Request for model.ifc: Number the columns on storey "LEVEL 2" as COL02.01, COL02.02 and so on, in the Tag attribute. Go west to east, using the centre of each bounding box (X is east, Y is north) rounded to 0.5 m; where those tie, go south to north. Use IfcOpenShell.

First a look at what the model holds.

```python
import ifcopenshell
import ifcopenshell.util.element
import ifcopenshell.util.placement

model = ifcopenshell.open("model.ifc")
print(model.schema)
storey = next(s for s in model.by_type("IfcBuildingStorey") if s.Name == "LEVEL 2")
columns = [e for e in ifcopenshell.util.element.get_decomposition(storey) if e.is_a("IfcColumn")]
for e in sorted(columns, key=lambda e: e.id()):
    origin = ifcopenshell.util.placement.get_local_placement(e.ObjectPlacement)[:3, 3]
    print(e.id(), e.Tag, e.Name, origin.round(2) + 0.0, sep=" | ")
```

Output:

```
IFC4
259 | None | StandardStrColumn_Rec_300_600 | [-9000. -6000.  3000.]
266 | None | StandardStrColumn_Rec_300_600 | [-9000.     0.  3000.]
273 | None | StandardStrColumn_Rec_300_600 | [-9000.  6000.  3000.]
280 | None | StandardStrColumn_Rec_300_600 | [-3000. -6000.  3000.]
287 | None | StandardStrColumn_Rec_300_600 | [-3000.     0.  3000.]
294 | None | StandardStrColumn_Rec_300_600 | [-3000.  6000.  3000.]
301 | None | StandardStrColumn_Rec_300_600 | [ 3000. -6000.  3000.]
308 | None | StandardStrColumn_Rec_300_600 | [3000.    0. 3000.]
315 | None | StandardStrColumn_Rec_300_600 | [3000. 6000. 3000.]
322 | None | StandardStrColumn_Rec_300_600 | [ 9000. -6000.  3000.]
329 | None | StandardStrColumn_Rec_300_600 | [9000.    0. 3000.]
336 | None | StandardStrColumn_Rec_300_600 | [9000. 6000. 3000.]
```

```python
import ifcopenshell
import ifcopenshell.geom
import ifcopenshell.util.element
import ifcopenshell.util.shape

model = ifcopenshell.open("model.ifc")
settings = ifcopenshell.geom.settings()
settings.set("use-world-coords", True)


def centre(element):
    shape = ifcopenshell.geom.create_shape(settings, element)
    return ifcopenshell.util.shape.get_bbox_centroid(shape.geometry)


storey = next(s for s in model.by_type("IfcBuildingStorey") if s.Name == "LEVEL 2")
columns = [e for e in ifcopenshell.util.element.get_decomposition(storey) if e.is_a("IfcColumn")]

# Insertion points can sit at a corner or the storey origin, so sort by the geometry (in metres).
centres = {e: centre(e) for e in columns}
columns.sort(key=lambda e: (round(centres[e][0] / 0.5), centres[e][1]))

for i, e in enumerate(columns, start=1):
    number = f"COL02.{i:02d}"
    e.Tag = number
    print(e.id(), number)

model.write("model-out.ifc")
```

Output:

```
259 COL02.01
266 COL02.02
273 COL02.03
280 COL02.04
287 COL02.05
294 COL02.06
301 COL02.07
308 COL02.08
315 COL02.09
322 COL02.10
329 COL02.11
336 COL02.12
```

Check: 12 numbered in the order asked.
